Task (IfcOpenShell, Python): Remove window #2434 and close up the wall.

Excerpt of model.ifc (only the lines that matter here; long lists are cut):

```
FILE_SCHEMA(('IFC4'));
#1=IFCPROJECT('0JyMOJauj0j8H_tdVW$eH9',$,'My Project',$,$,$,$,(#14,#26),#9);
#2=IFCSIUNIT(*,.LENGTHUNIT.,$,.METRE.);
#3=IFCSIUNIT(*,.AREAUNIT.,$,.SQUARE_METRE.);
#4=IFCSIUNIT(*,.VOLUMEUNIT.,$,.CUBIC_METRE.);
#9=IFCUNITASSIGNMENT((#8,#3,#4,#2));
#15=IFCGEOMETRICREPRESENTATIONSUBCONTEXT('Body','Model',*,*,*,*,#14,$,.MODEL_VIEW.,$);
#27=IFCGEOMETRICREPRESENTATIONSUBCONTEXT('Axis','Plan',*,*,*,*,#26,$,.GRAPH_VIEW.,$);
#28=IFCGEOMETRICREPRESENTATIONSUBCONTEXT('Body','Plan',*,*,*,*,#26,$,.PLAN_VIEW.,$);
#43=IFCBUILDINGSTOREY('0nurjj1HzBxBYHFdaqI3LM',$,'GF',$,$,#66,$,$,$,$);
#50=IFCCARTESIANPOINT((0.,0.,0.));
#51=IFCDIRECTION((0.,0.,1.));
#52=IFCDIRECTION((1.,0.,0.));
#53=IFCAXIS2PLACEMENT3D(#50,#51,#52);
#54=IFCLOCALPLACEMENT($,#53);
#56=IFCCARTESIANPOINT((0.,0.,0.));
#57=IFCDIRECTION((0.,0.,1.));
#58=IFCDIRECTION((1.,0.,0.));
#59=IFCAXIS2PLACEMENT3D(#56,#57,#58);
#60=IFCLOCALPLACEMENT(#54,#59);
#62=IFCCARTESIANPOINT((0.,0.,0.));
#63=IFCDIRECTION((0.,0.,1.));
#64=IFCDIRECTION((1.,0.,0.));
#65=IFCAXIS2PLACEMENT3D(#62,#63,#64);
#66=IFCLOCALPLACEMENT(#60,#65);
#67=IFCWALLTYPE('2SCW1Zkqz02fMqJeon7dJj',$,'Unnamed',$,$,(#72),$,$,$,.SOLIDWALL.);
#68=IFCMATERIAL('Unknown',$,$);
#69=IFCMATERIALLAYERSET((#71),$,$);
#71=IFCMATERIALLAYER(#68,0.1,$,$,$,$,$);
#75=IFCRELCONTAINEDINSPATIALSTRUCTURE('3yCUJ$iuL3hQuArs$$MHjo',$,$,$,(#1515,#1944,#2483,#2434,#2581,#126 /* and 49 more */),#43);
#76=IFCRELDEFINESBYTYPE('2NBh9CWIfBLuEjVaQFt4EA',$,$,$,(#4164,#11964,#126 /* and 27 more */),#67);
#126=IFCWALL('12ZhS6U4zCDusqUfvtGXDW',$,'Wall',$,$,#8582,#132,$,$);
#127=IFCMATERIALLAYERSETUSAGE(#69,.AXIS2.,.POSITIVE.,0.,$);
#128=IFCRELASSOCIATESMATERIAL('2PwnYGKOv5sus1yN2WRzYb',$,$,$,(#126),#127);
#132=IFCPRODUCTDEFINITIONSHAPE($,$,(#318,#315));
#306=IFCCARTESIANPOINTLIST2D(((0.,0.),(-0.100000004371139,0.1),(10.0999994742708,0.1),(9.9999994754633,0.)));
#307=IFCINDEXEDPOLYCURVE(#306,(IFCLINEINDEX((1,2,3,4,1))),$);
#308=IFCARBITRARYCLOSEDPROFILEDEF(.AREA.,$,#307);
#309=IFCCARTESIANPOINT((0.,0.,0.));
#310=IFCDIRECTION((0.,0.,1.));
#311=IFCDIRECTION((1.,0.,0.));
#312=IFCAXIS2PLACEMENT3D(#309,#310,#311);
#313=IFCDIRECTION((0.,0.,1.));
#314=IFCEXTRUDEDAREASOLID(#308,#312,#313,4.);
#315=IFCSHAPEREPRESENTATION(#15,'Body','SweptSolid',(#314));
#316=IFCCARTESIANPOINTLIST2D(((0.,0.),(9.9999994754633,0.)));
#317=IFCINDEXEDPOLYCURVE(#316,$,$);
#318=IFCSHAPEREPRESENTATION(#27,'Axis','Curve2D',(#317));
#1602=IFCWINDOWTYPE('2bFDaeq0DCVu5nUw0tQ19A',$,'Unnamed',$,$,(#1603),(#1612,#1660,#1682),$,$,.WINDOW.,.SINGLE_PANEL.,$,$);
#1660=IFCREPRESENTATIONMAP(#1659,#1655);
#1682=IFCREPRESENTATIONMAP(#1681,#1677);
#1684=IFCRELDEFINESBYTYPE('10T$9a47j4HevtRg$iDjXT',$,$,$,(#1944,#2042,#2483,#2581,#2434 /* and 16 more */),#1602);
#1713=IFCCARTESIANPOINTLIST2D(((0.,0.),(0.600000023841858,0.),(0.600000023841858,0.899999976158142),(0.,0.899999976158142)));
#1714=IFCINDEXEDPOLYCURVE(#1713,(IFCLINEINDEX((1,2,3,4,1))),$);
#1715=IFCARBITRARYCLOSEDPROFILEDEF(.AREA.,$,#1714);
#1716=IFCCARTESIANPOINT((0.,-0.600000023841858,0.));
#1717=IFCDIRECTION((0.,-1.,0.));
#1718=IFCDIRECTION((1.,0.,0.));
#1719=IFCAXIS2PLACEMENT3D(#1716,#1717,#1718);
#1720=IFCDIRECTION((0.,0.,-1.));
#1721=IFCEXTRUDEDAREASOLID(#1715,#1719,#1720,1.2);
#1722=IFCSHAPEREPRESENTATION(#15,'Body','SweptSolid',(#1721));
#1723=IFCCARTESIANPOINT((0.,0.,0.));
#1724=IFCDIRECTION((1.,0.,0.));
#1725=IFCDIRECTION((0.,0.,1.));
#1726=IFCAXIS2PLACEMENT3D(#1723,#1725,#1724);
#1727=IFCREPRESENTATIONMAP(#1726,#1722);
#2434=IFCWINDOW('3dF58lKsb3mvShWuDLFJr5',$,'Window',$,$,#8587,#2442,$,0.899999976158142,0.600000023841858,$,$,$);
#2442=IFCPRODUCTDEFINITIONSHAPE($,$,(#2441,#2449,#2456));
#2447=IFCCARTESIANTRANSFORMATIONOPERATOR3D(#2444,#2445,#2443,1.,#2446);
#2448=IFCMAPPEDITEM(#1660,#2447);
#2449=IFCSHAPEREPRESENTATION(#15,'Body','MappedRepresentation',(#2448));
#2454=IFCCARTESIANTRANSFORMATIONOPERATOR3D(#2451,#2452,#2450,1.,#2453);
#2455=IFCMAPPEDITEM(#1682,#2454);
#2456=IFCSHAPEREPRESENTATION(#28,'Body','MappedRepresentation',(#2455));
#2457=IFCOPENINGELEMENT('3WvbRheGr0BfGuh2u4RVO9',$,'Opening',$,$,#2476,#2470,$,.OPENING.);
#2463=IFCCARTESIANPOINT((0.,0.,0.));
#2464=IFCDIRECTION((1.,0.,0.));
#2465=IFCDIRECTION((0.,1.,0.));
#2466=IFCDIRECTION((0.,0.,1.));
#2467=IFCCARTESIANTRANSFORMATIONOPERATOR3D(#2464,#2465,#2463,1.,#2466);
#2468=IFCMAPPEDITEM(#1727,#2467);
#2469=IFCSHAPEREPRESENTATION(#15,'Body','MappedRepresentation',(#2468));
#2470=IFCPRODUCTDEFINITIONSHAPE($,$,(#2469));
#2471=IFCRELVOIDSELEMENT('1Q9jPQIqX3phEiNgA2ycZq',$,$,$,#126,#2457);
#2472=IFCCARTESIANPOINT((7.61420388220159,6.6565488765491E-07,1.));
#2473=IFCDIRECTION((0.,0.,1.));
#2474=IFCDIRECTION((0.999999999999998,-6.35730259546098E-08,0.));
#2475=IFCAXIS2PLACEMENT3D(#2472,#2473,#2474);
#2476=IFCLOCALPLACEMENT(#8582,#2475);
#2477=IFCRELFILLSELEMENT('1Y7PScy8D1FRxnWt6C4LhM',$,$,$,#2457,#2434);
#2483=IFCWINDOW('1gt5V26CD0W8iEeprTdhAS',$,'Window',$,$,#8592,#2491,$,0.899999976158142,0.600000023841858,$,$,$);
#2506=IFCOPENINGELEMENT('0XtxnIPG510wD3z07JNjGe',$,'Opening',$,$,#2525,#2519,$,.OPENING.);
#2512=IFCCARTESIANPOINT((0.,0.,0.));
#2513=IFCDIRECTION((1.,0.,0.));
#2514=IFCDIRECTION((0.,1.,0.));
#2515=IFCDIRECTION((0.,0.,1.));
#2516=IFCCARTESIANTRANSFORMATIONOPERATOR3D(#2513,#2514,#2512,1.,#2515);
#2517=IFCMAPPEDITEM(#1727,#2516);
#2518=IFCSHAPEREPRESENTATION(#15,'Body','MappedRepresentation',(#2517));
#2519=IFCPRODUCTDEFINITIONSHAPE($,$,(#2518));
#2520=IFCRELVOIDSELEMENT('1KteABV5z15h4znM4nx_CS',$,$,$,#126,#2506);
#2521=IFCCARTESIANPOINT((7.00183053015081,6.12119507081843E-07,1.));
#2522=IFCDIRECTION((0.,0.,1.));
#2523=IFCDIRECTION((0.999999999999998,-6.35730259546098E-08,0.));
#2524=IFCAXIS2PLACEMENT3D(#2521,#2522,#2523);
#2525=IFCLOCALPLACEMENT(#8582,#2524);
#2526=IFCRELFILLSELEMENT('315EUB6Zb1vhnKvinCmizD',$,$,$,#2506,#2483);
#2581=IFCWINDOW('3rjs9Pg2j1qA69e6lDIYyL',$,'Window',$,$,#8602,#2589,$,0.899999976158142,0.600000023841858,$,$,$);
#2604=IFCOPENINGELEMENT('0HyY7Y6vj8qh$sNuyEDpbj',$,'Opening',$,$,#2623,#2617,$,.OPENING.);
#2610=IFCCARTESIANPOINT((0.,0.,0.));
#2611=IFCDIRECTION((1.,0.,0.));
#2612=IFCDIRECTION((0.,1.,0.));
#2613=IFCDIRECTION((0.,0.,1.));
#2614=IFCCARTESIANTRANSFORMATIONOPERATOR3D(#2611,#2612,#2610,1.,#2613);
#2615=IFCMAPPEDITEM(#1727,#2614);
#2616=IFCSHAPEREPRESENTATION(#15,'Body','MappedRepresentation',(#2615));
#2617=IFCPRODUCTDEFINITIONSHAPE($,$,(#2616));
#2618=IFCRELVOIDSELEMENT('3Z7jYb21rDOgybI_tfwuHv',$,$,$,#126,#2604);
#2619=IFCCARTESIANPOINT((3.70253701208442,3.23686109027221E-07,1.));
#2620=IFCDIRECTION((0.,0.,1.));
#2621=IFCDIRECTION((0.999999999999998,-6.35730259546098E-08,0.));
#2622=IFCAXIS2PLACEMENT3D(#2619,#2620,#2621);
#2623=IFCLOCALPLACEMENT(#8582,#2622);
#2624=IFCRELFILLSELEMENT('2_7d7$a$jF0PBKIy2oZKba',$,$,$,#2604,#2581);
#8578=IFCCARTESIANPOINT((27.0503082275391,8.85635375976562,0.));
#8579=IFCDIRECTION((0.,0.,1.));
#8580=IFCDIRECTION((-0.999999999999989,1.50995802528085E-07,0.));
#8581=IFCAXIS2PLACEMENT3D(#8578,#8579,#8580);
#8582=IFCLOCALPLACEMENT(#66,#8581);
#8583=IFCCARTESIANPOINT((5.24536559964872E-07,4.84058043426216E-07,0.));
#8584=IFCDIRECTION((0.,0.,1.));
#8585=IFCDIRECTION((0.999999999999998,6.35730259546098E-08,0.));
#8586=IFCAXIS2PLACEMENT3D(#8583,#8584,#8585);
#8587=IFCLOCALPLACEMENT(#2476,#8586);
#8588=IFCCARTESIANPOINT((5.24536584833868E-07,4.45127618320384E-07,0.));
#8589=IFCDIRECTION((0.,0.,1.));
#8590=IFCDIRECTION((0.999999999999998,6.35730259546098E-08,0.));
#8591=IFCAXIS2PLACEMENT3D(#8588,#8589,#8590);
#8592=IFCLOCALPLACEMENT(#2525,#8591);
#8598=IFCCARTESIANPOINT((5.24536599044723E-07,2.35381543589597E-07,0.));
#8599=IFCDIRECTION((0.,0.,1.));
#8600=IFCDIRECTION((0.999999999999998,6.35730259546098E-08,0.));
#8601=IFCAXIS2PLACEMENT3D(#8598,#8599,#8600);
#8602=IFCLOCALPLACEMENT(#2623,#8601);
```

```python
import ifcopenshell
import ifcopenshell.api.feature
import ifcopenshell.api.root
import ifcopenshell.geom
import ifcopenshell.util.shape

model = ifcopenshell.open("model.ifc")
settings = ifcopenshell.geom.settings()


def volume(element):
    """Net volume in cubic metres, openings subtracted."""
    shape = ifcopenshell.geom.create_shape(settings, element)
    return ifcopenshell.util.shape.get_volume(shape.geometry)


window = model.by_guid("3dF58lKsb3mvShWuDLFJr5")
opening = window.FillsVoids[0].RelatingOpeningElement
wall = opening.VoidsElements[0].RelatingBuildingElement
before = volume(wall)

ifcopenshell.api.root.remove_product(model, product=window)
ifcopenshell.api.feature.remove_feature(model, feature=opening)

after = volume(wall)

print(f"wall volume {before:.3f} -> {after:.3f} m3")

model.write("model_v2.ifc")
```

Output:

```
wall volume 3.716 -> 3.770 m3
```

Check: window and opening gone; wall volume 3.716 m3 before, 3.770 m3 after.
